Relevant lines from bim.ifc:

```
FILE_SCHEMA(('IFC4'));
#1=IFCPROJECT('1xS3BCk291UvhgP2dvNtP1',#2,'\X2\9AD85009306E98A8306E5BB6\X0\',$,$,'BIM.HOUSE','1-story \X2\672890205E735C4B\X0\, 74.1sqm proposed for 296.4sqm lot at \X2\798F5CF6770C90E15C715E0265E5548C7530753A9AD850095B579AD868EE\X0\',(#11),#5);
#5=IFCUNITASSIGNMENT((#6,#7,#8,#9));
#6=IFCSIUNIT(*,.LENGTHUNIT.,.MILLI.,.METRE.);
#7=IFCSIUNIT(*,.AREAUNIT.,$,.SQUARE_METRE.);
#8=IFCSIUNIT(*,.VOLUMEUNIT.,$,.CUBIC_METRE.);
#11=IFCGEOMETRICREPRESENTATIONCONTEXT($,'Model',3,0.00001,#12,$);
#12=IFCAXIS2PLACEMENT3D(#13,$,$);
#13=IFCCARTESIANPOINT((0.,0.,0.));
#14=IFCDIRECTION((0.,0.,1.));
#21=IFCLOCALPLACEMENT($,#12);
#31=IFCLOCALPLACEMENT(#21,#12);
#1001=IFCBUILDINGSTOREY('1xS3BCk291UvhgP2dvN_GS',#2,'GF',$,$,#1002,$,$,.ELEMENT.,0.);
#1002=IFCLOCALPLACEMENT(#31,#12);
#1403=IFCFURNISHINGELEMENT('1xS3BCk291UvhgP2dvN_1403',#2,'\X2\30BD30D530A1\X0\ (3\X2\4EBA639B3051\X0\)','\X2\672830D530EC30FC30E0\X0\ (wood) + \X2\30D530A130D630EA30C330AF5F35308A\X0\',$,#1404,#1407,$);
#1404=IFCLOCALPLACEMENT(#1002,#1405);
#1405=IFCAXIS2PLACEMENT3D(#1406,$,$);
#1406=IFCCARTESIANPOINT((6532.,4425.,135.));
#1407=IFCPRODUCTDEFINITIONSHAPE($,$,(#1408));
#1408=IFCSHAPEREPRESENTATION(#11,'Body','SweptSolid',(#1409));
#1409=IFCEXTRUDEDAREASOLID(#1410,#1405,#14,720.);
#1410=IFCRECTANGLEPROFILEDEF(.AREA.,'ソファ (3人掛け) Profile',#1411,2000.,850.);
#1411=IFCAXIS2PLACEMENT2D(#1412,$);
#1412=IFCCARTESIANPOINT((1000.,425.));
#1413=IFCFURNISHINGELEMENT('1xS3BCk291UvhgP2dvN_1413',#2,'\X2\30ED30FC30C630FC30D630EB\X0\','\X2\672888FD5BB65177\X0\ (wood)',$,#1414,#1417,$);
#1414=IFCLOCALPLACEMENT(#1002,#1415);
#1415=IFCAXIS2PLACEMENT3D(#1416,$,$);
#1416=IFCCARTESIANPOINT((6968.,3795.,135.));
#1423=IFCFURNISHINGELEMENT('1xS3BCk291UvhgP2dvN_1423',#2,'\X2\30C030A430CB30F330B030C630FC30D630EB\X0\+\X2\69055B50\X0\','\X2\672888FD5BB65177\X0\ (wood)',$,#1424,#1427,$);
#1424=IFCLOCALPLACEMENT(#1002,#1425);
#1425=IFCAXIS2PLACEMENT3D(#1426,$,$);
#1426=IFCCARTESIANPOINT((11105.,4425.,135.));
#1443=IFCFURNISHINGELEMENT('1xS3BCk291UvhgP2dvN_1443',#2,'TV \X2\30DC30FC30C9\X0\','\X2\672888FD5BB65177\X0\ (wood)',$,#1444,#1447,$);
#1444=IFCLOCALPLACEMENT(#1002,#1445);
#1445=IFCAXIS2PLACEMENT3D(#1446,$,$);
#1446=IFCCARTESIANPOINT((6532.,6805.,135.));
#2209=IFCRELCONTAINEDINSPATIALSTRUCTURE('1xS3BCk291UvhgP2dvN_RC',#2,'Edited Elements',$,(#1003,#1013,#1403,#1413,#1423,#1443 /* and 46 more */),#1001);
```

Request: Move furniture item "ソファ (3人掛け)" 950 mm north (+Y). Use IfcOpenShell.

```python
import ifcopenshell
import ifcopenshell.api.geometry
import ifcopenshell.util.placement

model = ifcopenshell.open("bim.ifc")

item = model.by_id(1403)
matrix = ifcopenshell.util.placement.get_local_placement(item.ObjectPlacement)
matrix[1, 3] += 950.0
ifcopenshell.api.geometry.edit_object_placement(model, product=item, matrix=matrix, is_si=False)

print(ifcopenshell.util.placement.get_local_placement(item.ObjectPlacement).round(3) + 0.0)

model.write("bim_updated.ifc")
```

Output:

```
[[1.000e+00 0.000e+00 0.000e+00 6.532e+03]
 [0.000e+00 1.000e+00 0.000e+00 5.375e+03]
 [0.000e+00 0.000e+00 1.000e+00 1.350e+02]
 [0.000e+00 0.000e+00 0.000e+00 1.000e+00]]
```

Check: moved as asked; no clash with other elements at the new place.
